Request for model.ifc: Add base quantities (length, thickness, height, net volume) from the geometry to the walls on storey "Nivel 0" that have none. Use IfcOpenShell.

First a look at what the model holds.

```python
import ifcopenshell
import ifcopenshell.util.element
import ifcopenshell.util.unit

model = ifcopenshell.open("model.ifc")
print(model.schema)
for unit_type in ("LENGTHUNIT", "AREAUNIT", "VOLUMEUNIT"):
    print(unit_type, ifcopenshell.util.unit.calculate_unit_scale(model, unit_type))
storey = next(s for s in model.by_type("IfcBuildingStorey") if s.Name == "Nivel 0")
walls = [e for e in ifcopenshell.util.element.get_decomposition(storey) if e.is_a("IfcWall")]
for e in sorted(walls, key=lambda e: e.id()):
    print(e.id(), e.is_a(), e.Name, list(ifcopenshell.util.element.get_psets(e, qtos_only=True)), sep=" | ")
```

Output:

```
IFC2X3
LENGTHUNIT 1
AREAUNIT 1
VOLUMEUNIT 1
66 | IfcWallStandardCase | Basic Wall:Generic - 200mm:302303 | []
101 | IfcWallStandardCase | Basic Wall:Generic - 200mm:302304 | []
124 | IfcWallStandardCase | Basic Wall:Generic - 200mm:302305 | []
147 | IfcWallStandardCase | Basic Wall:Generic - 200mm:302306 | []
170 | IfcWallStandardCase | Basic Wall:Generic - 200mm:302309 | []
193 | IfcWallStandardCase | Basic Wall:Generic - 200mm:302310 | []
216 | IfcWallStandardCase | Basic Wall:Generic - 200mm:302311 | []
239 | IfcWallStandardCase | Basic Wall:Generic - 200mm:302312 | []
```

```python
import ifcopenshell
import ifcopenshell.api.pset
import ifcopenshell.geom
import ifcopenshell.util.element
import ifcopenshell.util.shape
import ifcopenshell.util.unit

model = ifcopenshell.open("model.ifc")
unit_scale = ifcopenshell.util.unit.calculate_unit_scale(model)
volume_scale = ifcopenshell.util.unit.calculate_unit_scale(model, "VOLUMEUNIT")
settings = ifcopenshell.geom.settings()

storey = next(s for s in model.by_type("IfcBuildingStorey") if s.Name == "Nivel 0")
walls = [e for e in ifcopenshell.util.element.get_decomposition(storey) if e.is_a("IfcWall")]

for e in sorted(walls, key=lambda e: e.id()):
    if ifcopenshell.util.element.get_psets(e, qtos_only=True, should_inherit=False):
        continue
    # Geometry comes back in metres, in the element's own axes.
    shape = ifcopenshell.geom.create_shape(settings, e)
    values = {
        "Length": ifcopenshell.util.shape.get_x(shape.geometry) / unit_scale,
        "Width": ifcopenshell.util.shape.get_y(shape.geometry) / unit_scale,
        "Height": ifcopenshell.util.shape.get_z(shape.geometry) / unit_scale,
        "NetVolume": ifcopenshell.util.shape.get_volume(shape.geometry) / volume_scale,
    }
    qto = ifcopenshell.api.pset.add_qto(model, product=e, name="BaseQuantities")
    ifcopenshell.api.pset.edit_qto(model, qto=qto, properties=values)
    print(e.id(), {k: round(v, 3) for k, v in values.items()})

model.write("model_rev.ifc")
```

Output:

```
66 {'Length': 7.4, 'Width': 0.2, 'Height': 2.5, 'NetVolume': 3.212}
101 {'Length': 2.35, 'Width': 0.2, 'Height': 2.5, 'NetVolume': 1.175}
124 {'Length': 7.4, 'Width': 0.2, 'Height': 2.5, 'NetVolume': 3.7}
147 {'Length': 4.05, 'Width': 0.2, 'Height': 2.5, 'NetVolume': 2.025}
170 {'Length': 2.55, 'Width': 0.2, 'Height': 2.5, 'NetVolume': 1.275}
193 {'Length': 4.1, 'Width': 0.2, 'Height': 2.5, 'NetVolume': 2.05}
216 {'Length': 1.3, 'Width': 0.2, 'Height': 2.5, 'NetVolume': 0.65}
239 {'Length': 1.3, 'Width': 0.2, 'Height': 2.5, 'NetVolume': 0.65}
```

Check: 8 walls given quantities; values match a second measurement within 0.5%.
